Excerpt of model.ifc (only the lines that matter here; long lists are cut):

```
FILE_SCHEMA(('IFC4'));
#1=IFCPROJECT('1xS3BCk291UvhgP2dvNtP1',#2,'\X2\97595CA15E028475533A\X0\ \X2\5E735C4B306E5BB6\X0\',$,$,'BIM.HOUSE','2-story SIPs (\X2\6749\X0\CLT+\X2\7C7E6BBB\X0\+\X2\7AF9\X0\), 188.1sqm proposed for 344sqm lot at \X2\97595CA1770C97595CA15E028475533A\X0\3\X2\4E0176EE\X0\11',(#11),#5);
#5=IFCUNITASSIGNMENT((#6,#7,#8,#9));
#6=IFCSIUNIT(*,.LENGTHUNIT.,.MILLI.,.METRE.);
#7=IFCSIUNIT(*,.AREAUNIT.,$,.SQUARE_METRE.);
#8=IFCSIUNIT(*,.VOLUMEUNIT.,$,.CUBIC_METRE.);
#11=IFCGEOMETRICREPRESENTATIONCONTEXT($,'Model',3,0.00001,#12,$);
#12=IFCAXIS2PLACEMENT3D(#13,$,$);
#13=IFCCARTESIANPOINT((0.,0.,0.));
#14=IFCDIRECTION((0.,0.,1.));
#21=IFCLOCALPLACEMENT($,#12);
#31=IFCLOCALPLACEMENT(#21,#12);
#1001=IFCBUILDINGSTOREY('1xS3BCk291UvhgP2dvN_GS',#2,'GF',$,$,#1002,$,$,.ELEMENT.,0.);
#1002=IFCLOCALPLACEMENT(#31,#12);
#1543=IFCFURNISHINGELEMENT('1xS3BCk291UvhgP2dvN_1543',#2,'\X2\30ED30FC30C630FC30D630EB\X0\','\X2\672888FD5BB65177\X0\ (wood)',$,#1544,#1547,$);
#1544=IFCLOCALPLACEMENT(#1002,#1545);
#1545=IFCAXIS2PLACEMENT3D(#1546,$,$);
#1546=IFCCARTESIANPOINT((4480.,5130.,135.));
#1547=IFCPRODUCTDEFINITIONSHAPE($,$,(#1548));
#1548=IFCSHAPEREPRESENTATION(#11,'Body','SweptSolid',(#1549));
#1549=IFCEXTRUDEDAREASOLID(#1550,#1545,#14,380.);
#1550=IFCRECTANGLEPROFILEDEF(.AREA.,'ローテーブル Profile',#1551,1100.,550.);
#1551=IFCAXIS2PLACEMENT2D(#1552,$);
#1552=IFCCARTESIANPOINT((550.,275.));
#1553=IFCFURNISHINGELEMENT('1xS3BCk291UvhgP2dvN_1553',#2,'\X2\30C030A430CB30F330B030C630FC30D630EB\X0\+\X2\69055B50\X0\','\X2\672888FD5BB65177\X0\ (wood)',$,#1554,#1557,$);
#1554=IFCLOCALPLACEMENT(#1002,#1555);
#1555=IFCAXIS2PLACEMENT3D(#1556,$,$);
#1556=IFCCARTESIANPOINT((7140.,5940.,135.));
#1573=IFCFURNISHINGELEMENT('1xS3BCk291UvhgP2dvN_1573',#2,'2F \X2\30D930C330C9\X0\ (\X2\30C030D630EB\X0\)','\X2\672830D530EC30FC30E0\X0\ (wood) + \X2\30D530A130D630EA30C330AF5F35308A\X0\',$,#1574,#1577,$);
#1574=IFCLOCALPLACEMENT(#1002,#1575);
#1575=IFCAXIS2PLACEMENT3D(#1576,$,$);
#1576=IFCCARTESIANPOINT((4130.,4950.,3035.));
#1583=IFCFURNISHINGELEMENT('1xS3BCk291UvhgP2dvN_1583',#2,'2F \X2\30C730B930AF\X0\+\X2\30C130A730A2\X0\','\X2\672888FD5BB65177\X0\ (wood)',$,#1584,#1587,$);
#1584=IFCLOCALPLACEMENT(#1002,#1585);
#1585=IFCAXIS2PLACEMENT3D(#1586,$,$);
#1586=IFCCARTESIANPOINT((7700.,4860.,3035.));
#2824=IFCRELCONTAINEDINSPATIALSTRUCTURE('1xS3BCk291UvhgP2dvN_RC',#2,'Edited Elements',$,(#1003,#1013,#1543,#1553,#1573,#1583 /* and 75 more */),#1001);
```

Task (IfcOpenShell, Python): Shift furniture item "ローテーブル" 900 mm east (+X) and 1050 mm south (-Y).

```python
import ifcopenshell
import ifcopenshell.api.geometry
import ifcopenshell.util.placement

model = ifcopenshell.open("model.ifc")

item = model.by_id(1543)
matrix = ifcopenshell.util.placement.get_local_placement(item.ObjectPlacement)
matrix[0, 3] += 900.0
matrix[1, 3] -= 1050.0
ifcopenshell.api.geometry.edit_object_placement(model, product=item, matrix=matrix, is_si=False)

print(ifcopenshell.util.placement.get_local_placement(item.ObjectPlacement).round(3) + 0.0)

model.write("model_updated.ifc")
```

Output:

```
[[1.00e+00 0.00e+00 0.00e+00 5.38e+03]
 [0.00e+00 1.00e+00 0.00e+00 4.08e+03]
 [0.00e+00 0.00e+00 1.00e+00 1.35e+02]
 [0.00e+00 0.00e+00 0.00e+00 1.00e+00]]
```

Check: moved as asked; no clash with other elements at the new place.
